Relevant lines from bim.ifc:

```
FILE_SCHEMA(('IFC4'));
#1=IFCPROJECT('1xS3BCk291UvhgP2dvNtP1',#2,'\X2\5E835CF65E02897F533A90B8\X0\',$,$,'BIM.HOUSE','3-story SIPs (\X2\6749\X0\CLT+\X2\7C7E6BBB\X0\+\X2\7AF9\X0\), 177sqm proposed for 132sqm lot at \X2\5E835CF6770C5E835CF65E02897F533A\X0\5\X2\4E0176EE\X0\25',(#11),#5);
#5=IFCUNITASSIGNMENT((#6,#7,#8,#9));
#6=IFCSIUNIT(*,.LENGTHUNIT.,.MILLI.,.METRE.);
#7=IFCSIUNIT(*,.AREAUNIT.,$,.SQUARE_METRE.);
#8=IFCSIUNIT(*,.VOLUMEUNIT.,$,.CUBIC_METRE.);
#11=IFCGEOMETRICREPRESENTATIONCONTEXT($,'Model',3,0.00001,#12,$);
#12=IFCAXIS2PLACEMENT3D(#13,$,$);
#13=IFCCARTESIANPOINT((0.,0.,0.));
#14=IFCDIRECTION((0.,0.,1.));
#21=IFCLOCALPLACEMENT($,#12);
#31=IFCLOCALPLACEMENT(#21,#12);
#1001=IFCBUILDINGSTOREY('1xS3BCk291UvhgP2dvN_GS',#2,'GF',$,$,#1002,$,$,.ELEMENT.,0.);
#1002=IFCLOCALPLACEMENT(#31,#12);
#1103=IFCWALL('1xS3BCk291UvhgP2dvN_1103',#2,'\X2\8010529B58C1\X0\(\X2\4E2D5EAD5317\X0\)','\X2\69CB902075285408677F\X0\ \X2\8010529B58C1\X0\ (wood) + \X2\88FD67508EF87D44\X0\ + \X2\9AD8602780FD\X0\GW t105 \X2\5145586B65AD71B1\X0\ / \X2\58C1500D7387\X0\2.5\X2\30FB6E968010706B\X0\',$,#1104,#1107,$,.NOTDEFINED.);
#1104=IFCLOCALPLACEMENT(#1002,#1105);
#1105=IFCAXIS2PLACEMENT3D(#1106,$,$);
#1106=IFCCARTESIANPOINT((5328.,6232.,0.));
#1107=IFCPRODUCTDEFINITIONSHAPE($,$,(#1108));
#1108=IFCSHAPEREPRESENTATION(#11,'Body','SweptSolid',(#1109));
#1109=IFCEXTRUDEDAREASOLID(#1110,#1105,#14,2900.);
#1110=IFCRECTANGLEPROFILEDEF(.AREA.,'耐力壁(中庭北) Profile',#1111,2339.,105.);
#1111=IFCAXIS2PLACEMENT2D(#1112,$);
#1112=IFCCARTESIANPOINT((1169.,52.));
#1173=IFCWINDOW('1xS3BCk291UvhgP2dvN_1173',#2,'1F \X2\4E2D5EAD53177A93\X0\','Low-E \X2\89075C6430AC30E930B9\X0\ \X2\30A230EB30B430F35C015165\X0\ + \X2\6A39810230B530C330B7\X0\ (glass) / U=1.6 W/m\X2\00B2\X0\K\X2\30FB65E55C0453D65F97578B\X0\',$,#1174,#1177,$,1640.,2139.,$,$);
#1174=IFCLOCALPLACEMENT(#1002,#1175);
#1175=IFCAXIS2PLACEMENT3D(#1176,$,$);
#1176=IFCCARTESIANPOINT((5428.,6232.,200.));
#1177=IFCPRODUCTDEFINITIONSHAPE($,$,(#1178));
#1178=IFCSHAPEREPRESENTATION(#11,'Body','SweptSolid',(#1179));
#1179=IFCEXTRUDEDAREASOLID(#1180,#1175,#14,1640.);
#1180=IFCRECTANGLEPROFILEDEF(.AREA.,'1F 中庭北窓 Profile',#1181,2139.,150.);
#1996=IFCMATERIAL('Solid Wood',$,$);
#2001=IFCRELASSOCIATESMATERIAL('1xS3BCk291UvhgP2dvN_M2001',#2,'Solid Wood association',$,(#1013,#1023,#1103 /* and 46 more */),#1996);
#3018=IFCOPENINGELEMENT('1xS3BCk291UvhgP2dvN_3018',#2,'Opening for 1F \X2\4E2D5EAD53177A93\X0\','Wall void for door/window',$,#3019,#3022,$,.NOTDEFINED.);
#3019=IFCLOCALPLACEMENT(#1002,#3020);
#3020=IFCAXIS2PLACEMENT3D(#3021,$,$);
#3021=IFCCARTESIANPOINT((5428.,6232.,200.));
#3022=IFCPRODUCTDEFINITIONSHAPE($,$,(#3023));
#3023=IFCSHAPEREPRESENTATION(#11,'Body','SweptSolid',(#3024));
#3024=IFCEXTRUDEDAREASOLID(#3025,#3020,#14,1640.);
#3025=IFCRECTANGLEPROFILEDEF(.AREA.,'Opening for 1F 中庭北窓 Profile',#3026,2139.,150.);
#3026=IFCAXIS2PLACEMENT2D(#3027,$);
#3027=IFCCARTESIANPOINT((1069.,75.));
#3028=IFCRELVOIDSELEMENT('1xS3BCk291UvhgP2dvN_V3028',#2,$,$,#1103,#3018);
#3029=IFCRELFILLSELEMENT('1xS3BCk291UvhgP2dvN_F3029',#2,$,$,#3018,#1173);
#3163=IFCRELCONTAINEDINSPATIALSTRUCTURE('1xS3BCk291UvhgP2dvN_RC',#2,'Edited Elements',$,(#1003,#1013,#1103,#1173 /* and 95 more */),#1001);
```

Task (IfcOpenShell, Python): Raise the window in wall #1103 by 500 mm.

```python
import numpy as np
import ifcopenshell
import ifcopenshell.api.geometry
import ifcopenshell.util.placement
import ifcopenshell.util.unit

model = ifcopenshell.open("bim.ifc")
unit_scale = ifcopenshell.util.unit.calculate_unit_scale(model)

window = model.by_guid("1xS3BCk291UvhgP2dvN_1173")
opening = window.FillsVoids[0].RelatingOpeningElement
dz = 500.0

shift = np.array([0.0, 0.0, dz])
# The window is not placed relative to its opening, so move both.
for product in (opening, window):
    matrix = ifcopenshell.util.placement.get_local_placement(product.ObjectPlacement)
    matrix[:3, 3] += shift
    ifcopenshell.api.geometry.edit_object_placement(model, product=product, matrix=matrix, is_si=False)

print(f"moved by {dz * unit_scale:+.3f} m")

model.write("bim-out.ifc")
```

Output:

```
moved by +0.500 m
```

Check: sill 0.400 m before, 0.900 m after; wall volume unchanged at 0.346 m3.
